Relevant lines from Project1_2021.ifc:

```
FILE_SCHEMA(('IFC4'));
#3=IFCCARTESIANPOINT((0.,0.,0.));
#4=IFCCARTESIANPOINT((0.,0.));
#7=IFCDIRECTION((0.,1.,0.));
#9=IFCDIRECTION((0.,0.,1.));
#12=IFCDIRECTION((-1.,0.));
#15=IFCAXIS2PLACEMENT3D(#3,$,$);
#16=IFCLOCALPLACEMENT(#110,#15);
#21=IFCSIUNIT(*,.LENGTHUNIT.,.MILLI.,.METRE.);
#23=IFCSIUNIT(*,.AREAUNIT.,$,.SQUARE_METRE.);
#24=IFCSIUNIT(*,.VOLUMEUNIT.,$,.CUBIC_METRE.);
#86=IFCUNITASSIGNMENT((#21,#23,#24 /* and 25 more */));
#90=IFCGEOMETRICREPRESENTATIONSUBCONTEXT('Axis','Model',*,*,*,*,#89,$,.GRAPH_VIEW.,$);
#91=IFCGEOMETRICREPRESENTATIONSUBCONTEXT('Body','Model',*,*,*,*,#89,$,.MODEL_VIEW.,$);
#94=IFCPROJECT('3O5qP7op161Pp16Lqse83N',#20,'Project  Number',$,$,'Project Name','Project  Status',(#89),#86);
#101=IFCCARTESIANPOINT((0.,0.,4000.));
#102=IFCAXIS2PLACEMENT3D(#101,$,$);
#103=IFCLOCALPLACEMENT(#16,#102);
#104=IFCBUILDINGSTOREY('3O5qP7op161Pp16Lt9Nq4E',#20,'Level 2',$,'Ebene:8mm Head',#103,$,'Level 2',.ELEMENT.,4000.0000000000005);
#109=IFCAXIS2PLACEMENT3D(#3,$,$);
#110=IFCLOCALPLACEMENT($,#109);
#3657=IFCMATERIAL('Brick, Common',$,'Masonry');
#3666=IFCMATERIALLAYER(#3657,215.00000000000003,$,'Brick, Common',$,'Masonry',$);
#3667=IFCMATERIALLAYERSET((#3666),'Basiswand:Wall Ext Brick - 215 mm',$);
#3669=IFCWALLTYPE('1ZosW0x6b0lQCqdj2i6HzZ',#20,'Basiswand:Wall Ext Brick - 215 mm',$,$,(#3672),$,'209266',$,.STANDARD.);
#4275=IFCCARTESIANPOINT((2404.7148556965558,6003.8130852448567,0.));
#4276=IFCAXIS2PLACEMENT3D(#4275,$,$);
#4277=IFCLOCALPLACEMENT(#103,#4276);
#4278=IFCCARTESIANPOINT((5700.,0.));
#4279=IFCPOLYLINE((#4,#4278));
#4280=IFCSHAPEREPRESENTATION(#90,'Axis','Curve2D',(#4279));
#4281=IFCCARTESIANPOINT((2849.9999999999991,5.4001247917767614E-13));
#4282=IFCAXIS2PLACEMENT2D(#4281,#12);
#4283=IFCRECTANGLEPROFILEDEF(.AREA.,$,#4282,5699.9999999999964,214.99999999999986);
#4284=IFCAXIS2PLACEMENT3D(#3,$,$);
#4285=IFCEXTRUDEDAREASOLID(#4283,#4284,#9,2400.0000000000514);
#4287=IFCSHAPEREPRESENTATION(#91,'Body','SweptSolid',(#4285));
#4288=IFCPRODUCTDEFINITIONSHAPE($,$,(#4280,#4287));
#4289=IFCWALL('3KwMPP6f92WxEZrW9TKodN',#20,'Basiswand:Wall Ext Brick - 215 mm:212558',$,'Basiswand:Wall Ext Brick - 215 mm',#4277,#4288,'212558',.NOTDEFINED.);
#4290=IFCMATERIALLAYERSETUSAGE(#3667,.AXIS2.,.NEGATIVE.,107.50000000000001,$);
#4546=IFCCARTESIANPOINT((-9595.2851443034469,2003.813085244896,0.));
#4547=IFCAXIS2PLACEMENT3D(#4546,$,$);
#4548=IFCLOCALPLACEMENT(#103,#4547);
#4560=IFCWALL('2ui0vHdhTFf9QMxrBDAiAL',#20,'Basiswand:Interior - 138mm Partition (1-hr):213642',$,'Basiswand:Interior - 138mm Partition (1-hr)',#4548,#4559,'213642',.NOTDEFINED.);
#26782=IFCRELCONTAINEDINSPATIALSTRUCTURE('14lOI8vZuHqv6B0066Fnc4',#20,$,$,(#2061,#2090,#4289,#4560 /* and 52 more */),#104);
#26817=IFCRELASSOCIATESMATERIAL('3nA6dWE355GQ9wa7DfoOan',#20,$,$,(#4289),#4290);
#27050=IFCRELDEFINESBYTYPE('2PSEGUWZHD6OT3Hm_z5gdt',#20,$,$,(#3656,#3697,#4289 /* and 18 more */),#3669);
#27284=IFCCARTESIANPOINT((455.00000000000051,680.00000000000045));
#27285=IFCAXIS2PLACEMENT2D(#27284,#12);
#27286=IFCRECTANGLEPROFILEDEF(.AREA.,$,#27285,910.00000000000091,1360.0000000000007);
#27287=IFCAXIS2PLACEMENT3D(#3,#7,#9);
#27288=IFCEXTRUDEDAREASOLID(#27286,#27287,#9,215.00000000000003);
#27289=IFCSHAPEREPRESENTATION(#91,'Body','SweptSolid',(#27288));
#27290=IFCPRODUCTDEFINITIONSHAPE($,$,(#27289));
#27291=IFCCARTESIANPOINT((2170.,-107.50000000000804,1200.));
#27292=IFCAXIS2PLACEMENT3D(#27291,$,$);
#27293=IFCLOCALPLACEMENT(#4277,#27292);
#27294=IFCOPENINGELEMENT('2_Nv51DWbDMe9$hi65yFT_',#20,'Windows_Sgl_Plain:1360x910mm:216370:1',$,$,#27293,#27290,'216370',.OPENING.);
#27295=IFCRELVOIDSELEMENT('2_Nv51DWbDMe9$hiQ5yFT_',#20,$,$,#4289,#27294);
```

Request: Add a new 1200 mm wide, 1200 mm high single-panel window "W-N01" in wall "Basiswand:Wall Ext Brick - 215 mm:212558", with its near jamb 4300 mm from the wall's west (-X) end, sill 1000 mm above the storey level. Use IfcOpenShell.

```python
import numpy as np
import ifcopenshell
import ifcopenshell.api.feature
import ifcopenshell.api.geometry
import ifcopenshell.api.root
import ifcopenshell.api.spatial
import ifcopenshell.geom
import ifcopenshell.util.element
import ifcopenshell.util.placement
import ifcopenshell.util.representation
import ifcopenshell.util.shape
import ifcopenshell.util.unit

model = ifcopenshell.open("Project1_2021.ifc")
unit_scale = ifcopenshell.util.unit.calculate_unit_scale(model)
settings = ifcopenshell.geom.settings()


def volume(element):
    """Net volume in cubic metres, openings subtracted."""
    shape = ifcopenshell.geom.create_shape(settings, element)
    return ifcopenshell.util.shape.get_volume(shape.geometry)


wall = model.by_id(4289)
storey = ifcopenshell.util.element.get_container(wall, ifc_class="IfcBuildingStorey")
context = ifcopenshell.util.representation.get_context(model, "Model", "Body", "MODEL_VIEW")
before = volume(wall)

width, height, from_end, sill = 1.2, 1.2, 4.3, 1  # metres

# The wall runs along its own X axis, and the end named is its -X end.
wall_shape = ifcopenshell.geom.create_shape(settings, wall)
x, y, z = ifcopenshell.util.shape.get_vertices(wall_shape.geometry).T
start = x.min() + from_end
face, thickness = float(y.min()), float(y.max() - y.min())
wall_matrix = ifcopenshell.util.placement.get_local_placement(wall.ObjectPlacement)
level = ifcopenshell.util.placement.get_local_placement(storey.ObjectPlacement)[2, 3]


def in_wall(x, y):
    """Placement at x, y metres in the wall's axes, at sill height."""
    matrix = wall_matrix.copy()
    matrix[:, 3] = wall_matrix @ np.array([x / unit_scale, y / unit_scale, 0.0, 1.0])
    matrix[2, 3] = level + sill / unit_scale
    return matrix


# Opening: a box that overshoots both wall faces by 50 mm.
opening = ifcopenshell.api.root.create_entity(model, ifc_class="IfcOpeningElement", predefined_type="OPENING")
box = ifcopenshell.api.geometry.add_wall_representation(
    model, context=context, length=width, height=height, thickness=thickness + 0.1
)
ifcopenshell.api.geometry.assign_representation(model, product=opening, representation=box)
ifcopenshell.api.geometry.edit_object_placement(model, product=opening, matrix=in_wall(start, face - 0.05), is_si=False)
ifcopenshell.api.feature.add_feature(model, feature=opening, element=wall)

window = ifcopenshell.api.root.create_entity(model, ifc_class="IfcWindow", name="W-N01", predefined_type="WINDOW")
window.OverallWidth, window.OverallHeight = width / unit_scale, height / unit_scale
window.PartitioningType = "SINGLE_PANEL"
body = ifcopenshell.api.geometry.add_window_representation(
    model,
    context=context,
    overall_width=window.OverallWidth,
    overall_height=window.OverallHeight,
    partition_type="SINGLE_PANEL",
)
ifcopenshell.api.geometry.assign_representation(model, product=window, representation=body)
ifcopenshell.api.spatial.assign_container(model, products=[window], relating_structure=storey)
ifcopenshell.api.feature.add_filling(model, opening=opening, element=window)

# Centre the window in the wall's thickness.
ifcopenshell.api.geometry.edit_object_placement(model, product=window, matrix=in_wall(start, face), is_si=False)
window_shape = ifcopenshell.geom.create_shape(settings, window)
depth = ifcopenshell.util.shape.get_vertices(window_shape.geometry)[:, 1]
offset = face + thickness / 2 - (depth.min() + depth.max()) / 2
ifcopenshell.api.geometry.edit_object_placement(model, product=window, matrix=in_wall(start, offset), is_si=False)

after = volume(wall)

print(f"wall volume {before:.3f} -> {after:.3f} m3")

model.write("Project1_2021_updated.ifc")
```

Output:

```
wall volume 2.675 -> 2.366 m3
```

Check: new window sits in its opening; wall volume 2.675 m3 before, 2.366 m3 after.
